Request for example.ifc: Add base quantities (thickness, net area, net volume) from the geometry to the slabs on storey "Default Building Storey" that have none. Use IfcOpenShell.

First a look at what the model holds.

```python
import ifcopenshell
import ifcopenshell.util.element
import ifcopenshell.util.unit

model = ifcopenshell.open("example.ifc")
print(model.schema)
for unit_type in ("LENGTHUNIT", "AREAUNIT", "VOLUMEUNIT"):
    print(unit_type, ifcopenshell.util.unit.calculate_unit_scale(model, unit_type))
storey = next(s for s in model.by_type("IfcBuildingStorey") if s.Name == "Default Building Storey")
slabs = [e for e in ifcopenshell.util.element.get_decomposition(storey) if e.is_a("IfcSlab")]
for e in sorted(slabs, key=lambda e: e.id()):
    print(e.id(), e.is_a(), e.Name, list(ifcopenshell.util.element.get_psets(e, qtos_only=True)), sep=" | ")
```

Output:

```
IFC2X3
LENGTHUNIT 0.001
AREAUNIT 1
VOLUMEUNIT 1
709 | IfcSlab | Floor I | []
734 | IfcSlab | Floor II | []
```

```python
import ifcopenshell
import ifcopenshell.api.pset
import ifcopenshell.geom
import ifcopenshell.util.element
import ifcopenshell.util.shape
import ifcopenshell.util.unit

model = ifcopenshell.open("example.ifc")
unit_scale = ifcopenshell.util.unit.calculate_unit_scale(model)
area_scale = ifcopenshell.util.unit.calculate_unit_scale(model, "AREAUNIT")
volume_scale = ifcopenshell.util.unit.calculate_unit_scale(model, "VOLUMEUNIT")
settings = ifcopenshell.geom.settings()

storey = next(s for s in model.by_type("IfcBuildingStorey") if s.Name == "Default Building Storey")
slabs = [e for e in ifcopenshell.util.element.get_decomposition(storey) if e.is_a("IfcSlab")]

for e in sorted(slabs, key=lambda e: e.id()):
    if ifcopenshell.util.element.get_psets(e, qtos_only=True, should_inherit=False):
        continue
    # Geometry comes back in metres, in the element's own axes.
    shape = ifcopenshell.geom.create_shape(settings, e)
    values = {
        "Width": ifcopenshell.util.shape.get_z(shape.geometry) / unit_scale,
        "NetArea": ifcopenshell.util.shape.get_footprint_area(shape.geometry) / area_scale,
        "NetVolume": ifcopenshell.util.shape.get_volume(shape.geometry) / volume_scale,
    }
    qto = ifcopenshell.api.pset.add_qto(model, product=e, name="BaseQuantities")
    ifcopenshell.api.pset.edit_qto(model, qto=qto, properties=values)
    print(e.id(), {k: round(v, 3) for k, v in values.items()})

model.write("example_updated.ifc")
```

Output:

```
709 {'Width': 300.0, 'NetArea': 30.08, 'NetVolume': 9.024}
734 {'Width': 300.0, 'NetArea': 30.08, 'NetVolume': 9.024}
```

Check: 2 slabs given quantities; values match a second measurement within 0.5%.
